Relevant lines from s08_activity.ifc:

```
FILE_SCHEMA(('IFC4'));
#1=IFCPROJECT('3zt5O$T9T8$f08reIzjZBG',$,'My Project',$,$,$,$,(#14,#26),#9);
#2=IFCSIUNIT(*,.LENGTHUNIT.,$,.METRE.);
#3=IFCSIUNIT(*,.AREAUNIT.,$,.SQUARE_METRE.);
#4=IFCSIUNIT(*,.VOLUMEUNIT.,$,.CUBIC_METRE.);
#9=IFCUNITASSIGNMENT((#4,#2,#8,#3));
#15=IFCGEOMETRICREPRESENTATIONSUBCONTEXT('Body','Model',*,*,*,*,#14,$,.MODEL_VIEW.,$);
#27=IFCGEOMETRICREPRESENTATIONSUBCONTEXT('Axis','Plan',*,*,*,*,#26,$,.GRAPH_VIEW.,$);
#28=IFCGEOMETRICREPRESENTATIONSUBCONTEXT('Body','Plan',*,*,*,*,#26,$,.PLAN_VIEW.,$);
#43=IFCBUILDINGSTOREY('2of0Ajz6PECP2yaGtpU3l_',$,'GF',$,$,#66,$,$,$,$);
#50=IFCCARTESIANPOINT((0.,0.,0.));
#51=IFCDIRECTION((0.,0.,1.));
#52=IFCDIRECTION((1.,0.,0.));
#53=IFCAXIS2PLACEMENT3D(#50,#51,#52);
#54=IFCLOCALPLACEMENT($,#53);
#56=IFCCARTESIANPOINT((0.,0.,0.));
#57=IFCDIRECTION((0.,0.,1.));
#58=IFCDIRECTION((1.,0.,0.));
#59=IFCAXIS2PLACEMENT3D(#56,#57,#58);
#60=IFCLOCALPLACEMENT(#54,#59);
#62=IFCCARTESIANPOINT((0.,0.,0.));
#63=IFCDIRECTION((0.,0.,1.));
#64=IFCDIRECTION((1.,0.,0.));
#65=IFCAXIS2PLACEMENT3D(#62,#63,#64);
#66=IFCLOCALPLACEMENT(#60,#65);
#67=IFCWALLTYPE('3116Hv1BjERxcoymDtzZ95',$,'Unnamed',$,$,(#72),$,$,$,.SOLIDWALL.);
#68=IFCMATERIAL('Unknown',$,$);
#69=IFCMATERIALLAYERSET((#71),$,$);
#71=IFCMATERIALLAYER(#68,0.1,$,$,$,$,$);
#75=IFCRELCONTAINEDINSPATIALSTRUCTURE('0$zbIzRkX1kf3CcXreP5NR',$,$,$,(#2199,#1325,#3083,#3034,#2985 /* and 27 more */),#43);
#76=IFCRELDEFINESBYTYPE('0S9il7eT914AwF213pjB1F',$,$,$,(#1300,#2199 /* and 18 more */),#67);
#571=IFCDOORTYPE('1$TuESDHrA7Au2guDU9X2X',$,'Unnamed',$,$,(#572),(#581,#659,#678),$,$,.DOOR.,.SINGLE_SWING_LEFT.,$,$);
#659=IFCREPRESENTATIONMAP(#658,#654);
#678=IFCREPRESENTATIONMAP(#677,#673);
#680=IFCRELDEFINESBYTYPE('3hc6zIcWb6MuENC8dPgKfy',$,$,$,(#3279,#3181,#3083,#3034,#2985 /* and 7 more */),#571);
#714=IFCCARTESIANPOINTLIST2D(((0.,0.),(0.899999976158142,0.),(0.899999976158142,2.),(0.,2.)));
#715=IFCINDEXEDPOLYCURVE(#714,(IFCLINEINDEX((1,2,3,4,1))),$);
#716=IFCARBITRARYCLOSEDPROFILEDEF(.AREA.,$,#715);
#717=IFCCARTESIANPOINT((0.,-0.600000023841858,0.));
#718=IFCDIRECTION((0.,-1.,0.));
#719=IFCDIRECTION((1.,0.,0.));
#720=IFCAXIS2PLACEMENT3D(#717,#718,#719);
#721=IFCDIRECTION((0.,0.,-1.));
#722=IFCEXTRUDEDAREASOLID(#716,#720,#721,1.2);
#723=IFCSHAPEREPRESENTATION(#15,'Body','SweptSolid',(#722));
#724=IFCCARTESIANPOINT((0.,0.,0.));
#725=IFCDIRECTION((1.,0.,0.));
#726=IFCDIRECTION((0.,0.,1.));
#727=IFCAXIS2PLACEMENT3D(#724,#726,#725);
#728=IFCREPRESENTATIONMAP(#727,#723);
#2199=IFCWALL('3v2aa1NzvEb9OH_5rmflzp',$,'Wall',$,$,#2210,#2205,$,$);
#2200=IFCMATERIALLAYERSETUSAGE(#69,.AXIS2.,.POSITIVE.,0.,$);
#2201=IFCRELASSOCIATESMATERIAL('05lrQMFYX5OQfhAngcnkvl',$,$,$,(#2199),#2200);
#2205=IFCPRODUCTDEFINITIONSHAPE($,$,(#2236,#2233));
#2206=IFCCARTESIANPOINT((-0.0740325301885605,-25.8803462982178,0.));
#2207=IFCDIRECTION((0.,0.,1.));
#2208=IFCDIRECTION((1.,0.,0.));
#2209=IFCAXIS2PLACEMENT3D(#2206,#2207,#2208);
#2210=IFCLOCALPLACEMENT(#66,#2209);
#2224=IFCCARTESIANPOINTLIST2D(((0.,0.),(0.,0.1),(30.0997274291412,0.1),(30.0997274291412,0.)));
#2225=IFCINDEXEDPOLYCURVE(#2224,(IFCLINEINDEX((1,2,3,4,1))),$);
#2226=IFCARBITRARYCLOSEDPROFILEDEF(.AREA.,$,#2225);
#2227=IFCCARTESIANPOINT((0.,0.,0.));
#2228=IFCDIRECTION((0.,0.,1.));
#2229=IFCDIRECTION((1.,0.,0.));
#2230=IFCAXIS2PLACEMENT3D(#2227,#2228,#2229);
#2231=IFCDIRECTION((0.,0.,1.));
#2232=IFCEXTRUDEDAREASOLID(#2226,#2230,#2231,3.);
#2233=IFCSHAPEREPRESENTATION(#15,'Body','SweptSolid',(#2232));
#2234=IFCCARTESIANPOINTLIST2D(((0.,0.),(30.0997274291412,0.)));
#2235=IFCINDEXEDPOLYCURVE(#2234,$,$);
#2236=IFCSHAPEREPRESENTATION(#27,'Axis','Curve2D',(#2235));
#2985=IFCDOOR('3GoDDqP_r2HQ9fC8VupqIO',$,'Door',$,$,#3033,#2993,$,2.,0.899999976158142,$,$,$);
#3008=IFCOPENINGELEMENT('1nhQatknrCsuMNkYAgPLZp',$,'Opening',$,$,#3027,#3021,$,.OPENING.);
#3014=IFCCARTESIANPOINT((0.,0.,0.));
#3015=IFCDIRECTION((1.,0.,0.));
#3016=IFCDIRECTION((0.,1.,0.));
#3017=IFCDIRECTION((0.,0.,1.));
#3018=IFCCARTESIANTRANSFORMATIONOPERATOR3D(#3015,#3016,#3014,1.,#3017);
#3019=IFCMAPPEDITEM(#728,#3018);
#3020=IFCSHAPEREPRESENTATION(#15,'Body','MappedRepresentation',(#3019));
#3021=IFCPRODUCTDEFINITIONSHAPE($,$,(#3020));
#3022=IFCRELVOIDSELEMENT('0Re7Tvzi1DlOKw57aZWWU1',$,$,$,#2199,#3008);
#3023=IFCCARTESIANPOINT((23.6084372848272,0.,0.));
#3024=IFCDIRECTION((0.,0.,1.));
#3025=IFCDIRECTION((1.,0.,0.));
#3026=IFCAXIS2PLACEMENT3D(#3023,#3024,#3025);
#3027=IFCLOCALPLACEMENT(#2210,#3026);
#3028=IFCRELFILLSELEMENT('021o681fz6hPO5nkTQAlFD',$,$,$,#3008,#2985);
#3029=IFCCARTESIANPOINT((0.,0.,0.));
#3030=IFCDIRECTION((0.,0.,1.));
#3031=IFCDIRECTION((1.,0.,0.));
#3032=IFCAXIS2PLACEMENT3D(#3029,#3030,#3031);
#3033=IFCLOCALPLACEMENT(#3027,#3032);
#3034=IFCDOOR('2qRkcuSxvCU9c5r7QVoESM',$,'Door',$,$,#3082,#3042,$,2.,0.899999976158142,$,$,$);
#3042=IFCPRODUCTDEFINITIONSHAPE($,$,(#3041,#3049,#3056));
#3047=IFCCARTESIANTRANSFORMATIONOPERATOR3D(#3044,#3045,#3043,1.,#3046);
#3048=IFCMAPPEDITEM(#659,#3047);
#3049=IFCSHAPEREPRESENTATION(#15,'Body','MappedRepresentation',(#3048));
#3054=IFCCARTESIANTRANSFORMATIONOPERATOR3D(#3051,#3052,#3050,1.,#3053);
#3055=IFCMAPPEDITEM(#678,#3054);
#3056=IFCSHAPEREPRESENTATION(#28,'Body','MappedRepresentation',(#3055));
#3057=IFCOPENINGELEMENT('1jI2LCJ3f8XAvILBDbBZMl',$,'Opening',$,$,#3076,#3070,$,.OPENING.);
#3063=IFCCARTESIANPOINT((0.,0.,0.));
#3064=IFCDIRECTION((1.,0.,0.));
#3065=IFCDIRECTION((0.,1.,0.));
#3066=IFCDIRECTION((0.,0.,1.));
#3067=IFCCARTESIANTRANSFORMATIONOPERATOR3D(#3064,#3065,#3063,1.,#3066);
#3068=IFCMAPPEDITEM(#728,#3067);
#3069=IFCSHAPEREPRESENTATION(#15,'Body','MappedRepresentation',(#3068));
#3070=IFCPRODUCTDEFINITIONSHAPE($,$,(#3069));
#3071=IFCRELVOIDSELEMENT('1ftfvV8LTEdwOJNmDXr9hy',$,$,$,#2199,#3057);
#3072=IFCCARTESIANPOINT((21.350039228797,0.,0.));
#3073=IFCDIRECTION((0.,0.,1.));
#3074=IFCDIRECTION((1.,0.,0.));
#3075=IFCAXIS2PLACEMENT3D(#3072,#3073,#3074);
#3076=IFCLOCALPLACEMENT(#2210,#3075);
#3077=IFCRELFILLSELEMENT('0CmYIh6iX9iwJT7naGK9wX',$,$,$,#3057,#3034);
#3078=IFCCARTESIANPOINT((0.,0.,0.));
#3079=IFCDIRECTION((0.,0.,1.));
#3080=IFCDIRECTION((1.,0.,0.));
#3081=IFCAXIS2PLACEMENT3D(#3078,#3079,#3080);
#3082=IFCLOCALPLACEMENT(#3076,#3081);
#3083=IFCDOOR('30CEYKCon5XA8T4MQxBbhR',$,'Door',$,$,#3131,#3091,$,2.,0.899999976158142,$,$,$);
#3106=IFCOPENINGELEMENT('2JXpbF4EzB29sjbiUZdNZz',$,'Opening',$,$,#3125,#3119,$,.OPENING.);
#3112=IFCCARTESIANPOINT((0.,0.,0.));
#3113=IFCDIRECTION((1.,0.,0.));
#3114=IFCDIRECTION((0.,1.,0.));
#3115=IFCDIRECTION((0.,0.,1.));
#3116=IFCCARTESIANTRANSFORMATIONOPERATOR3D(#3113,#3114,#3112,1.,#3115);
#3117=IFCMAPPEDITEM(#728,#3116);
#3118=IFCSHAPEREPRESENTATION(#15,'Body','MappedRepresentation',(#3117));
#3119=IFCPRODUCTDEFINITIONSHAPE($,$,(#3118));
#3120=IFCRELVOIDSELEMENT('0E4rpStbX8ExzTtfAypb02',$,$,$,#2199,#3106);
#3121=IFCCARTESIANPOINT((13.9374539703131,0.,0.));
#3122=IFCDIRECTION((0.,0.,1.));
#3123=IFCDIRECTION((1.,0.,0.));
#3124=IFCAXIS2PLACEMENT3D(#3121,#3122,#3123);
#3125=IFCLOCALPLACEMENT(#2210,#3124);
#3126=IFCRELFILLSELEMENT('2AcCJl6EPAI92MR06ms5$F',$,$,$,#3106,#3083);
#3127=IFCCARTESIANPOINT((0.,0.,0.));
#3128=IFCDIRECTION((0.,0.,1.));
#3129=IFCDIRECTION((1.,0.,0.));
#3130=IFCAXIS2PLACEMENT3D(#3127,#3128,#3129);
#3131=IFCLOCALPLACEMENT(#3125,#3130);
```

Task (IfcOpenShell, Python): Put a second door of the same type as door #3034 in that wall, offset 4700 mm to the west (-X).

```python
import ifcopenshell
import ifcopenshell.api.feature
import ifcopenshell.api.geometry
import ifcopenshell.api.root
import ifcopenshell.geom
import ifcopenshell.util.element
import ifcopenshell.util.placement
import ifcopenshell.util.shape
import ifcopenshell.util.unit

model = ifcopenshell.open("s08_activity.ifc")
unit_scale = ifcopenshell.util.unit.calculate_unit_scale(model)
settings = ifcopenshell.geom.settings()


def volume(element):
    """Net volume in cubic metres, openings subtracted."""
    shape = ifcopenshell.geom.create_shape(settings, element)
    return ifcopenshell.util.shape.get_volume(shape.geometry)


door = model.by_guid("2qRkcuSxvCU9c5r7QVoESM")
opening = door.FillsVoids[0].RelatingOpeningElement
wall = opening.VoidsElements[0].RelatingBuildingElement
before = volume(wall)
shift = ifcopenshell.util.placement.get_local_placement(wall.ObjectPlacement)[:3, 0] * -4.7 / unit_scale

# copy_class copies the void relationship, type, container and properties, but no geometry.
new_opening = ifcopenshell.api.root.copy_class(model, product=opening)
new_opening.Representation = ifcopenshell.util.element.copy_deep(
    model, opening.Representation, exclude=["IfcGeometricRepresentationContext", "IfcRepresentationMap"]
)
new_door = ifcopenshell.api.root.copy_class(model, product=door)
new_door.Representation = ifcopenshell.util.element.copy_deep(
    model, door.Representation, exclude=["IfcGeometricRepresentationContext", "IfcRepresentationMap"]
)
ifcopenshell.api.feature.add_filling(model, opening=new_opening, element=new_door)

for old, new in ((opening, new_opening), (door, new_door)):
    matrix = ifcopenshell.util.placement.get_local_placement(old.ObjectPlacement)
    matrix[:3, 3] += shift
    ifcopenshell.api.geometry.edit_object_placement(model, product=new, matrix=matrix, is_si=False)

after = volume(wall)

print(f"wall volume {before:.3f} -> {after:.3f} m3")

model.write("s08_activity-out.ifc")
```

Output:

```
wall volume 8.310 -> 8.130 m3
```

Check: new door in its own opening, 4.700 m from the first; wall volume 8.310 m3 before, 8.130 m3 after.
